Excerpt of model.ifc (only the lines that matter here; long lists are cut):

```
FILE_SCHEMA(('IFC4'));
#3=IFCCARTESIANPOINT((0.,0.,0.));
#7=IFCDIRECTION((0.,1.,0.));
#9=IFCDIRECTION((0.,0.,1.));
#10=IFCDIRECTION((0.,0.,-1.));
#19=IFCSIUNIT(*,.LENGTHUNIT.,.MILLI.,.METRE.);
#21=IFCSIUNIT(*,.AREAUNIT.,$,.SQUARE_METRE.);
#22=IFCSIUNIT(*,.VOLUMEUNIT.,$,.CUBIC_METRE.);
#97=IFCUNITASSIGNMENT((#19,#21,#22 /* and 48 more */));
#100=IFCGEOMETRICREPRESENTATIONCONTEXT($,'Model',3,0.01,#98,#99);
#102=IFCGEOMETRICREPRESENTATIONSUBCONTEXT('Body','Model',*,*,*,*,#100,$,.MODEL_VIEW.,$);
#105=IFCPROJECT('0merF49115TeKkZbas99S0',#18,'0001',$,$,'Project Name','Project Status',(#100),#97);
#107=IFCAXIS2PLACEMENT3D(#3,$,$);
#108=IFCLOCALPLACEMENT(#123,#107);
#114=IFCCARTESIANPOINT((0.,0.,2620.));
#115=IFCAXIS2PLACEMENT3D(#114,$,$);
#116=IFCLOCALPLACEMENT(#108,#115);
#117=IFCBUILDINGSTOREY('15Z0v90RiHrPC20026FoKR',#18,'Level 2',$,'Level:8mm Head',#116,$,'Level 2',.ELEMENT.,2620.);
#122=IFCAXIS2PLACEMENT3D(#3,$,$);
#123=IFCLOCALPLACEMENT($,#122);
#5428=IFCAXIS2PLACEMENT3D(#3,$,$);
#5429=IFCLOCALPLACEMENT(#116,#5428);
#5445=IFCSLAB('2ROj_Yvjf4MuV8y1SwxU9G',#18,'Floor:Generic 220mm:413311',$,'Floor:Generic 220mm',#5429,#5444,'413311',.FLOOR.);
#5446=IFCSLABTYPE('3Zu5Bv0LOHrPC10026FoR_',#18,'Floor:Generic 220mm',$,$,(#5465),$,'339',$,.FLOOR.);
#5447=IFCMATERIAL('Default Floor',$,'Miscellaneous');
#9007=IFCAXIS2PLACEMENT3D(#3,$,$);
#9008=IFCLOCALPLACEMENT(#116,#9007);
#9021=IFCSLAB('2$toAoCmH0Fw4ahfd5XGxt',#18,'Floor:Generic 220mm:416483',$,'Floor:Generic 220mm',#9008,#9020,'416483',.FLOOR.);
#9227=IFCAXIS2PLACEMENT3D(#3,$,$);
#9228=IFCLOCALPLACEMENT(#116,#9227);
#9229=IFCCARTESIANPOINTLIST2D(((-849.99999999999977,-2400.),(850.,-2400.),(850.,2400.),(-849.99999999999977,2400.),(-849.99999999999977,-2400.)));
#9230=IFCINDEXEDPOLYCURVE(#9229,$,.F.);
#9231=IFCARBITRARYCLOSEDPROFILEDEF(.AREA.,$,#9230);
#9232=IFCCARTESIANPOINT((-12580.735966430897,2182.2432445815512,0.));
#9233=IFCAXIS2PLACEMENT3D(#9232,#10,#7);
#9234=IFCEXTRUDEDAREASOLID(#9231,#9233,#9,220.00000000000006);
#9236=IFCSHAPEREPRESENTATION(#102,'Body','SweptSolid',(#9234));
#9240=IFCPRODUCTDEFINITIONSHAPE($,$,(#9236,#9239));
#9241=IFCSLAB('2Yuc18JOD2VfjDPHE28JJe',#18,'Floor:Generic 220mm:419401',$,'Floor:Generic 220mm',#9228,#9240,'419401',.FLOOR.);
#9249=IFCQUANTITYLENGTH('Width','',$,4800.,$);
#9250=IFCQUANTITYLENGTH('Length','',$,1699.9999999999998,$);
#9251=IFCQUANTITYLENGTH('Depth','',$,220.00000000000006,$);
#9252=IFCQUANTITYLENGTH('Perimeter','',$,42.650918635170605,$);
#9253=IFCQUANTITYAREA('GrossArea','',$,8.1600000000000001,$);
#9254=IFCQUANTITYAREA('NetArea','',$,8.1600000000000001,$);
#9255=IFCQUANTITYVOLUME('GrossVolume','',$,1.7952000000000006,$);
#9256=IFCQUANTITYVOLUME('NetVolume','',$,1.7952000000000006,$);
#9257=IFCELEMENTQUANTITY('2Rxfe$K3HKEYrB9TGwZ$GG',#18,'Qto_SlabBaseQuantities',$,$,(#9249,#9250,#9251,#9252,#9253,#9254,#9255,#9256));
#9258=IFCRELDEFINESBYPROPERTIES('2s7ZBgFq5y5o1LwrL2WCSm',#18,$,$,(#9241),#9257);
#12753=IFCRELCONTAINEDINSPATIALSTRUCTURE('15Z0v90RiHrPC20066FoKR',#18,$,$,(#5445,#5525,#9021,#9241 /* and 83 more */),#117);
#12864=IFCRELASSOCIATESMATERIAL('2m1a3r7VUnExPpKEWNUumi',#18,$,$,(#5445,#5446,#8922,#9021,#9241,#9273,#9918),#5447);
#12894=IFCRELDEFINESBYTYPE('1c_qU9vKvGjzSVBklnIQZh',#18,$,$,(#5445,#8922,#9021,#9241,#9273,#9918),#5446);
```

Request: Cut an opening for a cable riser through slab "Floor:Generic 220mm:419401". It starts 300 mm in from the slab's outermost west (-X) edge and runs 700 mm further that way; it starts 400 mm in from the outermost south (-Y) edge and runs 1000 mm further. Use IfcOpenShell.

```python
import numpy as np
import ifcopenshell
import ifcopenshell.api.feature
import ifcopenshell.api.geometry
import ifcopenshell.api.pset
import ifcopenshell.api.root
import ifcopenshell.geom
import ifcopenshell.util.element
import ifcopenshell.util.placement
import ifcopenshell.util.representation
import ifcopenshell.util.shape
import ifcopenshell.util.unit

model = ifcopenshell.open("model.ifc")
unit_scale = ifcopenshell.util.unit.calculate_unit_scale(model)
area_scale = ifcopenshell.util.unit.calculate_unit_scale(model, "AREAUNIT")
volume_scale = ifcopenshell.util.unit.calculate_unit_scale(model, "VOLUMEUNIT")
settings = ifcopenshell.geom.settings()


def volume(element):
    """Net volume in cubic metres, openings subtracted."""
    shape = ifcopenshell.geom.create_shape(settings, element)
    return ifcopenshell.util.shape.get_volume(shape.geometry)


slab = model.by_guid("2Yuc18JOD2VfjDPHE28JJe")
before = volume(slab)

# Extent in the slab's own axes, in metres. The edges named are its -X and -Y sides.
slab_shape = ifcopenshell.geom.create_shape(settings, slab)
vertices = ifcopenshell.util.shape.get_vertices(slab_shape.geometry)
x_min, y_min, bottom = vertices.min(axis=0)
top = vertices[:, 2].max()

opening = ifcopenshell.api.root.create_entity(model, ifc_class="IfcOpeningElement", name="Cable riser opening", predefined_type="OPENING")
context = ifcopenshell.util.representation.get_context(model, "Model", "Body", "MODEL_VIEW")
width, depth = 0.7, 1
outline = [(0.0, 0.0), (width, 0.0), (width, depth), (0.0, depth), (0.0, 0.0)]
# Overshoot both faces by 50 mm so the cut is clean.
shape = ifcopenshell.api.geometry.add_slab_representation(
    model, context=context, depth=top - bottom + 0.1, polyline=outline
)
ifcopenshell.api.geometry.assign_representation(model, product=opening, representation=shape)

matrix = ifcopenshell.util.placement.get_local_placement(slab.ObjectPlacement)
matrix[:, 3] = matrix @ np.append(np.array([x_min + 0.3, y_min + 0.4, bottom - 0.05]) / unit_scale, 1.0)
ifcopenshell.api.geometry.edit_object_placement(model, product=opening, matrix=matrix, is_si=False)
ifcopenshell.api.feature.add_feature(model, feature=opening, element=slab)

after = volume(slab)

# Update the slab's stored quantities.
qto = model.by_id(ifcopenshell.util.element.get_pset(slab, "Qto_SlabBaseQuantities", should_inherit=False)["id"])
ifcopenshell.api.pset.edit_qto(model, qto=qto, properties={
    "NetArea": after / (top - bottom) / area_scale,
    "NetVolume": after / volume_scale,
})

print(f"slab volume {before:.3f} -> {after:.3f} m3")

model.write("model_rev.ifc")
```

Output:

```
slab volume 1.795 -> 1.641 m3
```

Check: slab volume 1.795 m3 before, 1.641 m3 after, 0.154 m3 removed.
